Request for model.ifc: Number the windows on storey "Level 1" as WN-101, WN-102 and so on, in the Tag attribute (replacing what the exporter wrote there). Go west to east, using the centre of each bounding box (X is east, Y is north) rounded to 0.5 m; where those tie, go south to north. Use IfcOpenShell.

First a look at what the model holds.

```python
import ifcopenshell
import ifcopenshell.util.element
import ifcopenshell.util.placement

model = ifcopenshell.open("model.ifc")
print(model.schema)
storey = next(s for s in model.by_type("IfcBuildingStorey") if s.Name == "Level 1")
windows = [e for e in ifcopenshell.util.element.get_decomposition(storey) if e.is_a("IfcWindow")]
for e in sorted(windows, key=lambda e: e.id()):
    origin = ifcopenshell.util.placement.get_local_placement(e.ObjectPlacement)[:3, 3]
    print(e.id(), e.Tag, e.Name, origin.round(2) + 0.0, sep=" | ")
```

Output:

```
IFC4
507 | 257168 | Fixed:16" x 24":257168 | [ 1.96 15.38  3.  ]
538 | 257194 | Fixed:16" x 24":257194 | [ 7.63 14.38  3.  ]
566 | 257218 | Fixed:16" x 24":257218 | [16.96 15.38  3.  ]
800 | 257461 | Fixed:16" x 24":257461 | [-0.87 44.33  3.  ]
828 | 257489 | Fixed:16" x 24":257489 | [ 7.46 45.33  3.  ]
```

```python
import ifcopenshell
import ifcopenshell.geom
import ifcopenshell.util.element
import ifcopenshell.util.shape

model = ifcopenshell.open("model.ifc")
settings = ifcopenshell.geom.settings()
settings.set("use-world-coords", True)


def centre(element):
    shape = ifcopenshell.geom.create_shape(settings, element)
    return ifcopenshell.util.shape.get_bbox_centroid(shape.geometry)


storey = next(s for s in model.by_type("IfcBuildingStorey") if s.Name == "Level 1")
windows = [e for e in ifcopenshell.util.element.get_decomposition(storey) if e.is_a("IfcWindow")]

# Insertion points can sit at a corner or the storey origin, so sort by the geometry (in metres).
centres = {e: centre(e) for e in windows}
windows.sort(key=lambda e: (round(centres[e][0] / 0.5), centres[e][1]))

for i, e in enumerate(windows, start=1):
    number = f"WN-1{i:02d}"
    e.Tag = number
    print(e.id(), number)

model.write("model_edited.ifc")
```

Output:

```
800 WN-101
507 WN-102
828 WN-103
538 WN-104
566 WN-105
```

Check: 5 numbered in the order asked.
